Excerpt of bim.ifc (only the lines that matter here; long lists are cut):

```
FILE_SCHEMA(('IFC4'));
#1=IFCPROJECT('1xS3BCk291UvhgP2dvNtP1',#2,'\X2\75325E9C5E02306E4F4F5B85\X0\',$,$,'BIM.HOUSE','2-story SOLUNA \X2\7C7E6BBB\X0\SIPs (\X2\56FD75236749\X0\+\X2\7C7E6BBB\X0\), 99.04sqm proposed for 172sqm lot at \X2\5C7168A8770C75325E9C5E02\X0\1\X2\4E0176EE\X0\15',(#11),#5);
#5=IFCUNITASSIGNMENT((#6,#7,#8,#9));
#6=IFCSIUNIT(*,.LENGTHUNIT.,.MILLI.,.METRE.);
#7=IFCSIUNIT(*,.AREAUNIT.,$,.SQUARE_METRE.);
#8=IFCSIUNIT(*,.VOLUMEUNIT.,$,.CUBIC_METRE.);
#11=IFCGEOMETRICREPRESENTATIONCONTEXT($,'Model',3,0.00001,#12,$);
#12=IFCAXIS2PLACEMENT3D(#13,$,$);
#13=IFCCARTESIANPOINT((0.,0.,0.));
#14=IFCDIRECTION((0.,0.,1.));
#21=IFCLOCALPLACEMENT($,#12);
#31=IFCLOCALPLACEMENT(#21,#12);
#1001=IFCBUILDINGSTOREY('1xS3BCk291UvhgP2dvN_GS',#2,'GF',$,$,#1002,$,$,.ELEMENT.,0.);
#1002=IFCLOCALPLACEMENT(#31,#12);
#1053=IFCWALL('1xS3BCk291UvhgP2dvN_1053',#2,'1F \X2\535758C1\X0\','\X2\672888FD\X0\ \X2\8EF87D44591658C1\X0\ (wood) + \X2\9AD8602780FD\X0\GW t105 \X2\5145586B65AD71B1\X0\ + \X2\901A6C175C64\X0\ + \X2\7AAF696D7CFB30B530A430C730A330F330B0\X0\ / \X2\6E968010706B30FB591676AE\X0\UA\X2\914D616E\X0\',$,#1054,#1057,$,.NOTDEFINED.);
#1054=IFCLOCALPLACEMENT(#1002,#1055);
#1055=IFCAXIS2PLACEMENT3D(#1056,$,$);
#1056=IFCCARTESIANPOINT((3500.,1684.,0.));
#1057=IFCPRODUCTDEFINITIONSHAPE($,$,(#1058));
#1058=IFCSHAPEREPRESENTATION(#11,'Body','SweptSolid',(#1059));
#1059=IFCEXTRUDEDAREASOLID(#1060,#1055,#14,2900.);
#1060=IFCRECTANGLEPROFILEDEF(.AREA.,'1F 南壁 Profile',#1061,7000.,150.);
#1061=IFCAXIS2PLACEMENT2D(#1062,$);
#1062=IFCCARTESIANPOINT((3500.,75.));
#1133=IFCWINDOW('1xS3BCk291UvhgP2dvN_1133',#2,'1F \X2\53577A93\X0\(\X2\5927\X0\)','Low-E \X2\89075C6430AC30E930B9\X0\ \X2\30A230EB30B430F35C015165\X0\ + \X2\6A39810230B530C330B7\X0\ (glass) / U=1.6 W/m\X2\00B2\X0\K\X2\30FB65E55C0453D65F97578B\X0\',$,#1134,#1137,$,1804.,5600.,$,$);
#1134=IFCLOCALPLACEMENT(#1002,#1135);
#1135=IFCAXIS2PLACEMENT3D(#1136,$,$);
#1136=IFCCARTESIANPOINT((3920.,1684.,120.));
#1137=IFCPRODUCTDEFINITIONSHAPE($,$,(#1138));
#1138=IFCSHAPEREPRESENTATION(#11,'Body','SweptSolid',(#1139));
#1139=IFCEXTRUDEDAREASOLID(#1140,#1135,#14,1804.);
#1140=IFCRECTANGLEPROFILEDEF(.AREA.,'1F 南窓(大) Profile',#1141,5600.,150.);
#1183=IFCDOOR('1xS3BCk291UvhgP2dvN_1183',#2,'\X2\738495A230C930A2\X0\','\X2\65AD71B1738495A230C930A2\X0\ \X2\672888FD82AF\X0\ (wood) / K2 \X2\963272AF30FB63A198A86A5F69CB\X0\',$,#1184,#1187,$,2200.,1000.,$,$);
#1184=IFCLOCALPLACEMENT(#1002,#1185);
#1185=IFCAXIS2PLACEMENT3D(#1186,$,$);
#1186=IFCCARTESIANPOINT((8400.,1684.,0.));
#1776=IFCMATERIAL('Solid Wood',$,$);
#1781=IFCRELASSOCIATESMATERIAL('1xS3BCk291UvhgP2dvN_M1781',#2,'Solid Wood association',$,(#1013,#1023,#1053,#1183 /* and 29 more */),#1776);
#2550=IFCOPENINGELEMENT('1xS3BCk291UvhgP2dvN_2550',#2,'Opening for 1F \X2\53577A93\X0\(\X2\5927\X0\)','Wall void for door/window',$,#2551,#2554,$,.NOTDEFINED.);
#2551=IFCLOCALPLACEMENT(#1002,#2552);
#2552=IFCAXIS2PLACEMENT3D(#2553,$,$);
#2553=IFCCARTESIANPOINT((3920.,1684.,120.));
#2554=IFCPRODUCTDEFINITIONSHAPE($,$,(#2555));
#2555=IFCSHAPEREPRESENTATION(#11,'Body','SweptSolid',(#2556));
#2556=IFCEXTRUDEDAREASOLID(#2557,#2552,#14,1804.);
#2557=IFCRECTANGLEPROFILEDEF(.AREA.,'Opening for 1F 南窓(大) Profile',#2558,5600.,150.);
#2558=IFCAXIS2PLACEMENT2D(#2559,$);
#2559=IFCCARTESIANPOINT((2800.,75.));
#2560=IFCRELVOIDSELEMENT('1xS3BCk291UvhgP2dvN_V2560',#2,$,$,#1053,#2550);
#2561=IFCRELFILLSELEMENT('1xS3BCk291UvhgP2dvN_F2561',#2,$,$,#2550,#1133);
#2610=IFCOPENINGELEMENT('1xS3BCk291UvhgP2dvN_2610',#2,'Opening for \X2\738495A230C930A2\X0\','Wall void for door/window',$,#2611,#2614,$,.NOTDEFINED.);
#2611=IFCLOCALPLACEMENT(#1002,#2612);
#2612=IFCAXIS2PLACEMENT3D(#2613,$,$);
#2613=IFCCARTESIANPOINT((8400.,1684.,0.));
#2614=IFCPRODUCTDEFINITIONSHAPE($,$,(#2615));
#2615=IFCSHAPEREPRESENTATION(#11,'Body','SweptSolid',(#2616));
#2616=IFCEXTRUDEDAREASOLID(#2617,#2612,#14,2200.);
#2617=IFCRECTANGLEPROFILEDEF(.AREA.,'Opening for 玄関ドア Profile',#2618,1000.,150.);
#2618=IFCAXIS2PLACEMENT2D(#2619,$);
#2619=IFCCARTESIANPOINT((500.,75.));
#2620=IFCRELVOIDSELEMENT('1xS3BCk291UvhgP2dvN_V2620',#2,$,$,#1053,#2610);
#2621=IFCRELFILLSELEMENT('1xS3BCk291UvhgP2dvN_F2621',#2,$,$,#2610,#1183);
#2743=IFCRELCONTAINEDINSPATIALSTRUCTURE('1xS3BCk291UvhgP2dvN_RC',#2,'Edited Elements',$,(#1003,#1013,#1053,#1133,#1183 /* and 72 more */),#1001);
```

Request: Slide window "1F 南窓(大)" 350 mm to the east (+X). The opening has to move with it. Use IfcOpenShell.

```python
import ifcopenshell
import ifcopenshell.api.geometry
import ifcopenshell.util.placement

model = ifcopenshell.open("bim.ifc")

window = model.by_id(1133)
opening = window.FillsVoids[0].RelatingOpeningElement
wall = opening.VoidsElements[0].RelatingBuildingElement

wall_matrix = ifcopenshell.util.placement.get_local_placement(wall.ObjectPlacement)
shift = wall_matrix[:3, 0] * 350.0
before = ifcopenshell.util.placement.get_local_placement(window.ObjectPlacement)[:3, 3].copy()

# The window is not placed relative to its opening, so move both.
for product in (opening, window):
    matrix = ifcopenshell.util.placement.get_local_placement(product.ObjectPlacement)
    matrix[:3, 3] += shift
    ifcopenshell.api.geometry.edit_object_placement(model, product=product, matrix=matrix, is_si=False)

after = ifcopenshell.util.placement.get_local_placement(window.ObjectPlacement)[:3, 3]
print("window moved by", (after - before).round(3) + 0.0)

model.write("bim_rev.ifc")
```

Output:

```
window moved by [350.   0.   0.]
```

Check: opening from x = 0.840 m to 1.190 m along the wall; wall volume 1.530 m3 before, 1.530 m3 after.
